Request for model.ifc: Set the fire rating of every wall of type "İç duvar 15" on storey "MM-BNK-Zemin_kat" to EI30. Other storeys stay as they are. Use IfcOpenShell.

First a look at what the model holds.

```python
import ifcopenshell
import ifcopenshell.util.element

model = ifcopenshell.open("model.ifc")
print(model.schema)
storey = next(s for s in model.by_type("IfcBuildingStorey") if s.Name == "MM-BNK-Zemin_kat")
walls = [e for e in ifcopenshell.util.element.get_decomposition(storey) if e.is_a("IfcWall")]
seen = {}
for e in walls:
    element_type = ifcopenshell.util.element.get_type(e)
    key = (element_type.Name if element_type != e and element_type else None, ifcopenshell.util.element.get_pset(e, "Pset_WallCommon", "FireRating"))
    seen[key] = seen.get(key, 0) + 1
for (name, value), count in sorted(seen.items(), key=str):
    print(count, "x", name, "|", value)
```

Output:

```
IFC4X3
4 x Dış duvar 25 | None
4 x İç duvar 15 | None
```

```python
import ifcopenshell
import ifcopenshell.api.pset
import ifcopenshell.util.element

model = ifcopenshell.open("model.ifc")

storey = next(s for s in model.by_type("IfcBuildingStorey") if s.Name == "MM-BNK-Zemin_kat")
walls = [e for e in ifcopenshell.util.element.get_decomposition(storey) if e.is_a("IfcWall")]

count = 0
for e in walls:
    element_type = ifcopenshell.util.element.get_type(e)
    if element_type in (None, e) or element_type.Name != "İç duvar 15":
        continue
    # add_pset returns the element's existing set when there is one.
    pset = ifcopenshell.api.pset.add_pset(model, product=e, name="Pset_WallCommon")
    ifcopenshell.api.pset.edit_pset(model, pset=pset, properties={"FireRating": "EI30"})
    count += 1

print(count, "walls updated")

model.write("model_edited.ifc")
```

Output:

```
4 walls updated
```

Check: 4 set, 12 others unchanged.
